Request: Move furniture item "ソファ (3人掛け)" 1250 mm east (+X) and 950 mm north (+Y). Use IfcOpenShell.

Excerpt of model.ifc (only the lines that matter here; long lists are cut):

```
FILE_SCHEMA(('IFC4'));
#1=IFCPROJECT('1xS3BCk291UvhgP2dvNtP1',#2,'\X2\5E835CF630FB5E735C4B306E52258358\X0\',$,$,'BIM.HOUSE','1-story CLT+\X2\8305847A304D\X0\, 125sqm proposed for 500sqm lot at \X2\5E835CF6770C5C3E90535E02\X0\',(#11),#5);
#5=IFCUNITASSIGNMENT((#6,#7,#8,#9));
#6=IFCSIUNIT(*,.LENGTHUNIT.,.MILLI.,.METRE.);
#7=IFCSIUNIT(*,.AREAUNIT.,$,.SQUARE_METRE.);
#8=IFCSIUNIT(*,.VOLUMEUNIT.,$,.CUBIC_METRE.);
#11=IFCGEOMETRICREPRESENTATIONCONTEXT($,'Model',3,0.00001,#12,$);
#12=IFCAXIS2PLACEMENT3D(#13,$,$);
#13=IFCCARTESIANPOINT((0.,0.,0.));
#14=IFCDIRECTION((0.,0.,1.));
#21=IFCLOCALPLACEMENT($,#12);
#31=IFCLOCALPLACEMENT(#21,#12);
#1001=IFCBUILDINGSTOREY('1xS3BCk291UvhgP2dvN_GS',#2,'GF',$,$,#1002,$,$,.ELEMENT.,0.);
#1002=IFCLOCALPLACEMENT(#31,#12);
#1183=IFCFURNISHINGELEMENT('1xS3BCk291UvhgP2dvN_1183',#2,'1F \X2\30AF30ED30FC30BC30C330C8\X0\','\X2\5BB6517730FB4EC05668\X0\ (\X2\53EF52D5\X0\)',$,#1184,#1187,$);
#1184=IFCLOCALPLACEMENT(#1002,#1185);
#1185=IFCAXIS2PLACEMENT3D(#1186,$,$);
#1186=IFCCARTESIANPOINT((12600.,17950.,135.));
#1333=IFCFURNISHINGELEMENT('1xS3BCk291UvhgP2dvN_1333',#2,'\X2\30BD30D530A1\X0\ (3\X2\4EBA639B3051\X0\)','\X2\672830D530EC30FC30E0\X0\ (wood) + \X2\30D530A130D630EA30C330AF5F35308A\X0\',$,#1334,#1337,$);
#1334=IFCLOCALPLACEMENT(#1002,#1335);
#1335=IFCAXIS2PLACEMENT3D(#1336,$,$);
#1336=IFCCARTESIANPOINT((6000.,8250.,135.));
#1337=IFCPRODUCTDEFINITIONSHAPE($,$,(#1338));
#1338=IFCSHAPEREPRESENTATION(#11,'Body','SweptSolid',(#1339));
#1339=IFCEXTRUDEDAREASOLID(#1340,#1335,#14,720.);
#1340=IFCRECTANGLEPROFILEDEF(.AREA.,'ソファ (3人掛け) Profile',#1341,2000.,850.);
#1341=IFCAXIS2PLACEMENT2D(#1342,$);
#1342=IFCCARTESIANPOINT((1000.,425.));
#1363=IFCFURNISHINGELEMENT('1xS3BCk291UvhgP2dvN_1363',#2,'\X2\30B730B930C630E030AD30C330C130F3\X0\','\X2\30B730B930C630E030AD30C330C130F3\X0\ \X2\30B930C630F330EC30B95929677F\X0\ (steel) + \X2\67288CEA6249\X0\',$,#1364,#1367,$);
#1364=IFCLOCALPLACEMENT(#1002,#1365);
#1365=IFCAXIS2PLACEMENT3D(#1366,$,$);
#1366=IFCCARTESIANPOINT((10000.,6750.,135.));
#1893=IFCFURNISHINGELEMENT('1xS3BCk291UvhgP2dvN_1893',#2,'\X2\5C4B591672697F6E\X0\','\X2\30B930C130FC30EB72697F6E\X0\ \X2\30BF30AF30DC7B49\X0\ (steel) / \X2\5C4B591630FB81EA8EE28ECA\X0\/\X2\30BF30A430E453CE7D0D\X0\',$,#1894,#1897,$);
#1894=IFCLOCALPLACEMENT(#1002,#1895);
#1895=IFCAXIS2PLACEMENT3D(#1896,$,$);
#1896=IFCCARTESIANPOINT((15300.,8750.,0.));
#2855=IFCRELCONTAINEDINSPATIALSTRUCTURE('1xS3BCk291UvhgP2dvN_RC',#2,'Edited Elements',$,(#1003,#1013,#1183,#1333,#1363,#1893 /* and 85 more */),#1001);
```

```python
import ifcopenshell
import ifcopenshell.api.geometry
import ifcopenshell.util.placement

model = ifcopenshell.open("model.ifc")

item = model.by_guid("1xS3BCk291UvhgP2dvN_1333")
matrix = ifcopenshell.util.placement.get_local_placement(item.ObjectPlacement)
matrix[0, 3] += 1250.0
matrix[1, 3] += 950.0
ifcopenshell.api.geometry.edit_object_placement(model, product=item, matrix=matrix, is_si=False)

print(ifcopenshell.util.placement.get_local_placement(item.ObjectPlacement).round(3) + 0.0)

model.write("model_updated.ifc")
```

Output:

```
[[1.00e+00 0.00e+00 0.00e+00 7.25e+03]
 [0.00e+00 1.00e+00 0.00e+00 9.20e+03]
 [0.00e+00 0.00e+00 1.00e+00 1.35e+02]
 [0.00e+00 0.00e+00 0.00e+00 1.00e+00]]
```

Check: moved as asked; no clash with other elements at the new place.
